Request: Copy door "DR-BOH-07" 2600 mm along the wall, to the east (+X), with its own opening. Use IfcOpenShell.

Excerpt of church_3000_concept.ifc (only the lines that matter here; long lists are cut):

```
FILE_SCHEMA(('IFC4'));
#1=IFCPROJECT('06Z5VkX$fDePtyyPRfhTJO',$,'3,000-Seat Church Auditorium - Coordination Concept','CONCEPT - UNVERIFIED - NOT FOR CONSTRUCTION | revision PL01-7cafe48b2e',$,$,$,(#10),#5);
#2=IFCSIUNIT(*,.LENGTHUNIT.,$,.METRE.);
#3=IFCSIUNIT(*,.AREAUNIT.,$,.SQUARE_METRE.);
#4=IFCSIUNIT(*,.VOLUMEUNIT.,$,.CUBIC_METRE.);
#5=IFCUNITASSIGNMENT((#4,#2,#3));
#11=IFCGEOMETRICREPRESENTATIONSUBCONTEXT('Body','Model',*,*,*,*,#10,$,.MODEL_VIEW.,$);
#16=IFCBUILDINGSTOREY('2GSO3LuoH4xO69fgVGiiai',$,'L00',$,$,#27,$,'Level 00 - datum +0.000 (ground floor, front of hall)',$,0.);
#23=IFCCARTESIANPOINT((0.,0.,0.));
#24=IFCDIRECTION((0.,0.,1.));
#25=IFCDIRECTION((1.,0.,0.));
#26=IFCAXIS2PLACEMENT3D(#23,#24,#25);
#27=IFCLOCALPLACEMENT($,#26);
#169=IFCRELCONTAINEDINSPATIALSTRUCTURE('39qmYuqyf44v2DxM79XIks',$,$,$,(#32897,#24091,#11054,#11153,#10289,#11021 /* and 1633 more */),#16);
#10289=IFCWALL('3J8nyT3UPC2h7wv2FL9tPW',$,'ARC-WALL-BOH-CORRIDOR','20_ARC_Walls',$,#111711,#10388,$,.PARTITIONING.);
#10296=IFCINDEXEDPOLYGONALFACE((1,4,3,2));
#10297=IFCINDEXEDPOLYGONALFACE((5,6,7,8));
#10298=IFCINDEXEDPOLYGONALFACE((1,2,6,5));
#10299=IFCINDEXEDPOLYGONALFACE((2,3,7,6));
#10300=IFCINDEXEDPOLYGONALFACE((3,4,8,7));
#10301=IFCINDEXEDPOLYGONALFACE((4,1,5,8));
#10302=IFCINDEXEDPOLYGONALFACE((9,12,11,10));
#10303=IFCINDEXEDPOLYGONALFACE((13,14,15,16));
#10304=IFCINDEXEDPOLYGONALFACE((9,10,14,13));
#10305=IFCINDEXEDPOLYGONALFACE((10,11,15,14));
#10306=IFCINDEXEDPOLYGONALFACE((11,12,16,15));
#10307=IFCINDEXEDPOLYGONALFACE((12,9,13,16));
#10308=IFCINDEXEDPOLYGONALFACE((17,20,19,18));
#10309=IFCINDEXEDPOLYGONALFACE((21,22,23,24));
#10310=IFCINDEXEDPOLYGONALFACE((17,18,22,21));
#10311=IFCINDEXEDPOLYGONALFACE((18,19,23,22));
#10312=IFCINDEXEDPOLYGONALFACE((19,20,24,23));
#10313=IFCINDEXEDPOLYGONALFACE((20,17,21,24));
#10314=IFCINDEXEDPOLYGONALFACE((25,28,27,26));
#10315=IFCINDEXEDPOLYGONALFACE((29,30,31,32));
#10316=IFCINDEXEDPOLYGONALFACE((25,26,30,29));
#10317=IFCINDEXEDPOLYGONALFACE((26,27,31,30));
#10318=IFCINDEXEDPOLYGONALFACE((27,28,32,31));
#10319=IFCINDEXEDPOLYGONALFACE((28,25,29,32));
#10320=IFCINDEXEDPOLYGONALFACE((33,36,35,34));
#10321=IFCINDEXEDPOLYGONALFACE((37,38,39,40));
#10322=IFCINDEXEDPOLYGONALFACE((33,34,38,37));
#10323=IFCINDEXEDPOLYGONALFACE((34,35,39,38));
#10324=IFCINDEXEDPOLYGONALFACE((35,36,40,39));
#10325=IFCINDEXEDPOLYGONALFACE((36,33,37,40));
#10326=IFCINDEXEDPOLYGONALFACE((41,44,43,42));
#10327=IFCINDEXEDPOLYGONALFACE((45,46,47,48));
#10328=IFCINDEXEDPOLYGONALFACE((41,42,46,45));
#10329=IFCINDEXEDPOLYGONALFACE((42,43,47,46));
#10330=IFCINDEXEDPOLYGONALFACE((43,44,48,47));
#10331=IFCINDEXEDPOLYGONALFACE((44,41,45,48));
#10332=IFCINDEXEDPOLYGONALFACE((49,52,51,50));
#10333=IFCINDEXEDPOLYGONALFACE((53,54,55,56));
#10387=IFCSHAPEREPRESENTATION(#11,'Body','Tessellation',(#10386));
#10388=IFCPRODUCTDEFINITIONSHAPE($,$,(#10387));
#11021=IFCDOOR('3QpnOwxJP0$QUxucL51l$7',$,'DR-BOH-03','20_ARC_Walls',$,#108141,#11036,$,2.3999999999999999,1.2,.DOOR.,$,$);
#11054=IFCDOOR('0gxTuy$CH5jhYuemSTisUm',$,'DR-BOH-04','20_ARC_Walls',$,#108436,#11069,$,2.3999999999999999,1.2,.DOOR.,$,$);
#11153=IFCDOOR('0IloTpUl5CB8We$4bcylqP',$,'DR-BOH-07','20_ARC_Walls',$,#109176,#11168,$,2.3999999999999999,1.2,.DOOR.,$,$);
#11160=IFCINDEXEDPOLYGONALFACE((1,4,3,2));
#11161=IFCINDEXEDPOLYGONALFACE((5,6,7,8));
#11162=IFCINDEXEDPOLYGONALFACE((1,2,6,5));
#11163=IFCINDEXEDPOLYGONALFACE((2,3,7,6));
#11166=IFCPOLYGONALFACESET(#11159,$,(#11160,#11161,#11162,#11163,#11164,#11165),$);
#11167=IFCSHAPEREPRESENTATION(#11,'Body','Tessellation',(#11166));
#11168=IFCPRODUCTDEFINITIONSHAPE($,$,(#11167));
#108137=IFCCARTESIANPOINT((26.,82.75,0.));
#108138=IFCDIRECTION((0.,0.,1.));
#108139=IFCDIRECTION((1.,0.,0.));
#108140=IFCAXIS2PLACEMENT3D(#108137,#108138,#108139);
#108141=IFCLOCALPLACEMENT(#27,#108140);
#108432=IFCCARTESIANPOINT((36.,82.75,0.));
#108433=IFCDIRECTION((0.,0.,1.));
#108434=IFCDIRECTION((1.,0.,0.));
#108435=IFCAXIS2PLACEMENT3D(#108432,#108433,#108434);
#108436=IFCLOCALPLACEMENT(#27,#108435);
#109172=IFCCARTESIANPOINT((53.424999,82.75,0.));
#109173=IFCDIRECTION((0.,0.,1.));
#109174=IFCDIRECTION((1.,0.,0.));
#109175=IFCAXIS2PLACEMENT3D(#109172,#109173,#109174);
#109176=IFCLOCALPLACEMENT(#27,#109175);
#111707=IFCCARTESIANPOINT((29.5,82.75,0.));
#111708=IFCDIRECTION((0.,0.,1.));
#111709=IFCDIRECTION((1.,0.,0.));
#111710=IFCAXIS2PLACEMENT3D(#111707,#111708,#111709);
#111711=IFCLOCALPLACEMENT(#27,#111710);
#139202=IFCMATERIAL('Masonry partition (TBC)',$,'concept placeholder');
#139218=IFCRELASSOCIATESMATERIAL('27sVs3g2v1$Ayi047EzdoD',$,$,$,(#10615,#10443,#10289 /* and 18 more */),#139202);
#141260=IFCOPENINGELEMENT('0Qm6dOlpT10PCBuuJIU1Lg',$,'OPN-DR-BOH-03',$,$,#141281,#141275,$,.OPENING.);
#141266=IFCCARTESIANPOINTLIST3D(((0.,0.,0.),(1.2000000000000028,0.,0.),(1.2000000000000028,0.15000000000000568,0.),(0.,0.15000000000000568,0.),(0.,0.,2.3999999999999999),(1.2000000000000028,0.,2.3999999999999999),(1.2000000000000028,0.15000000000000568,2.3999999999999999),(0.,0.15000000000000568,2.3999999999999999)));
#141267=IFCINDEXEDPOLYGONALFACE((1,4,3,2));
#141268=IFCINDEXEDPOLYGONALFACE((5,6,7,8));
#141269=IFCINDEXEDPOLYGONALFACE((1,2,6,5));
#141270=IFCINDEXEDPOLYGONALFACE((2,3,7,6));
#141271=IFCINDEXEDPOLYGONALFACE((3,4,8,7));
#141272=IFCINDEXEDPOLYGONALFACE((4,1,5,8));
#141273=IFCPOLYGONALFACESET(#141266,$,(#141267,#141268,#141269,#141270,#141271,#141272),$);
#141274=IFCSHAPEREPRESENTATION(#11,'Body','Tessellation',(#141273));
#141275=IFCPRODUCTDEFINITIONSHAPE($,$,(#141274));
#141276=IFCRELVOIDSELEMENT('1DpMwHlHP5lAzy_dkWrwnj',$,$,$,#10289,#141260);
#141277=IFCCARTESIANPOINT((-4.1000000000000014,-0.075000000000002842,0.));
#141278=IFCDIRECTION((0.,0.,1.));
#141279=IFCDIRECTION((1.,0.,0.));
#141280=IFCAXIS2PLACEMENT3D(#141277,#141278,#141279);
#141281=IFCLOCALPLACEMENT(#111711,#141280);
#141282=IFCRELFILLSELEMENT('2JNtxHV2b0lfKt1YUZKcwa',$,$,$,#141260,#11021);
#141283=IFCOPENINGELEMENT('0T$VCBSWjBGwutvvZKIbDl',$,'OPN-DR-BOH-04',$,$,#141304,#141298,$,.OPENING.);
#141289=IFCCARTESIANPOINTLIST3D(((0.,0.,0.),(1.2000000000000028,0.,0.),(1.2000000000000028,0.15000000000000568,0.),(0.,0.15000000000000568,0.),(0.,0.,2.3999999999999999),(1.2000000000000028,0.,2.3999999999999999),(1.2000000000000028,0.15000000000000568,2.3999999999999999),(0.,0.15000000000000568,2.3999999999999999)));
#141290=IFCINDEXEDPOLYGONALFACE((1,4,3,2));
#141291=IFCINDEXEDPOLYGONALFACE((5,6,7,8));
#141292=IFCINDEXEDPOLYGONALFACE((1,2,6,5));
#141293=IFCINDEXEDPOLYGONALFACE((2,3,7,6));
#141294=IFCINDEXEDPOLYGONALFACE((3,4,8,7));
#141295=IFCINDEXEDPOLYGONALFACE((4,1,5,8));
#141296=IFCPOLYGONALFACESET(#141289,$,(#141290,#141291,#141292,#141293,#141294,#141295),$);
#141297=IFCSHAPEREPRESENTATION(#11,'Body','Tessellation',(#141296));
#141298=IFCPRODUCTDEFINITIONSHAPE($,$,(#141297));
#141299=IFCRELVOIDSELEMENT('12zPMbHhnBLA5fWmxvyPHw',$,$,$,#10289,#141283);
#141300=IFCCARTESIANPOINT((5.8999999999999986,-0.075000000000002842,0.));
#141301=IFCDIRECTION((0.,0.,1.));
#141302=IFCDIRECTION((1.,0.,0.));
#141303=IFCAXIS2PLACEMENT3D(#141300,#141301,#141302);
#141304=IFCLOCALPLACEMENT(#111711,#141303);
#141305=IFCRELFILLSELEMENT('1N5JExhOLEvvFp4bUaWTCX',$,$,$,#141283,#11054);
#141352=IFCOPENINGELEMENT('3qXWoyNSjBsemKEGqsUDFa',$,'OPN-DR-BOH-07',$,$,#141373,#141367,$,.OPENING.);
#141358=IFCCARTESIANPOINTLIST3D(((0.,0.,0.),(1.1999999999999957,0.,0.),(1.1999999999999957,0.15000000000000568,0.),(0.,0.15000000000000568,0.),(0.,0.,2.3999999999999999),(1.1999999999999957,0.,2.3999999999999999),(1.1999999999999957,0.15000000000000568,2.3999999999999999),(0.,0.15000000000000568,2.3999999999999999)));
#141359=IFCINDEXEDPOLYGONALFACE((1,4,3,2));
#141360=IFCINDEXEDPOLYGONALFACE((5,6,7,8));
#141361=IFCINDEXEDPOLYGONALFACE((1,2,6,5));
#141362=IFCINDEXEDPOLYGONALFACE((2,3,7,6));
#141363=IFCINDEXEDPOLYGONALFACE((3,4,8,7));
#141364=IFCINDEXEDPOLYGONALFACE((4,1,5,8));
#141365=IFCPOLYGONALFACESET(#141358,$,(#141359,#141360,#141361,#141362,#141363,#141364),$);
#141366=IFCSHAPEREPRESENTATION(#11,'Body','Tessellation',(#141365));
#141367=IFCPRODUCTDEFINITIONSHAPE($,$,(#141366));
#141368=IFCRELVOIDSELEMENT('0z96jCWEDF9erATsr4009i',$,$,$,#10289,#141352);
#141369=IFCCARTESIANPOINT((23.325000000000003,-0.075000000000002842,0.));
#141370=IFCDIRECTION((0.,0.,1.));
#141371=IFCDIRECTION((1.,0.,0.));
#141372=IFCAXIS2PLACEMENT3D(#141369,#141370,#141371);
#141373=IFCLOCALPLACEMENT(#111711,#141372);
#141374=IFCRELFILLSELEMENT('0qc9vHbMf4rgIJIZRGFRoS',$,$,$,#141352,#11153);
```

```python
import ifcopenshell
import ifcopenshell.api.feature
import ifcopenshell.api.geometry
import ifcopenshell.api.root
import ifcopenshell.geom
import ifcopenshell.util.element
import ifcopenshell.util.placement
import ifcopenshell.util.shape
import ifcopenshell.util.unit

model = ifcopenshell.open("church_3000_concept.ifc")
unit_scale = ifcopenshell.util.unit.calculate_unit_scale(model)
settings = ifcopenshell.geom.settings()


def volume(element):
    """Net volume in cubic metres, openings subtracted."""
    shape = ifcopenshell.geom.create_shape(settings, element)
    return ifcopenshell.util.shape.get_volume(shape.geometry)


door = model.by_guid("0IloTpUl5CB8We$4bcylqP")
opening = door.FillsVoids[0].RelatingOpeningElement
wall = opening.VoidsElements[0].RelatingBuildingElement
before = volume(wall)
shift = ifcopenshell.util.placement.get_local_placement(wall.ObjectPlacement)[:3, 0] * 2.6 / unit_scale

# copy_class copies the void relationship, type, container and properties, but no geometry.
new_opening = ifcopenshell.api.root.copy_class(model, product=opening)
new_opening.Representation = ifcopenshell.util.element.copy_deep(
    model, opening.Representation, exclude=["IfcGeometricRepresentationContext", "IfcRepresentationMap"]
)
new_door = ifcopenshell.api.root.copy_class(model, product=door)
new_door.Representation = ifcopenshell.util.element.copy_deep(
    model, door.Representation, exclude=["IfcGeometricRepresentationContext", "IfcRepresentationMap"]
)
ifcopenshell.api.feature.add_filling(model, opening=new_opening, element=new_door)

for old, new in ((opening, new_opening), (door, new_door)):
    matrix = ifcopenshell.util.placement.get_local_placement(old.ObjectPlacement)
    matrix[:3, 3] += shift
    ifcopenshell.api.geometry.edit_object_placement(model, product=new, matrix=matrix, is_si=False)

after = volume(wall)

print(f"wall volume {before:.3f} -> {after:.3f} m3")

model.write("church_3000_concept_rev.ifc")
```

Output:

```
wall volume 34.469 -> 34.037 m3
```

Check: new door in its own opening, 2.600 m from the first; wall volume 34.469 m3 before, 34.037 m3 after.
